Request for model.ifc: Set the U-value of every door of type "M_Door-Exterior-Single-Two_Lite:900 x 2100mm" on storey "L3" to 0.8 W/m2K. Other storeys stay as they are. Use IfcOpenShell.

First a look at what the model holds.

```python
import ifcopenshell
import ifcopenshell.util.element

model = ifcopenshell.open("model.ifc")
print(model.schema)
storey = next(s for s in model.by_type("IfcBuildingStorey") if s.Name == "L3")
doors = [e for e in ifcopenshell.util.element.get_decomposition(storey) if e.is_a("IfcDoor")]
seen = {}
for e in doors:
    element_type = ifcopenshell.util.element.get_type(e)
    key = (element_type.Name if element_type != e and element_type else None, ifcopenshell.util.element.get_pset(e, "Pset_DoorCommon", "ThermalTransmittance"))
    seen[key] = seen.get(key, 0) + 1
for (name, value), count in sorted(seen.items(), key=str):
    print(count, "x", name, "|", value)
```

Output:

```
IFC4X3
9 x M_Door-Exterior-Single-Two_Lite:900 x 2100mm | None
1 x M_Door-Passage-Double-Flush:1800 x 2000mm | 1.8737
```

```python
import ifcopenshell
import ifcopenshell.api.pset
import ifcopenshell.util.element

model = ifcopenshell.open("model.ifc")

storey = next(s for s in model.by_type("IfcBuildingStorey") if s.Name == "L3")
doors = [e for e in ifcopenshell.util.element.get_decomposition(storey) if e.is_a("IfcDoor")]

count = 0
for e in doors:
    element_type = ifcopenshell.util.element.get_type(e)
    if element_type in (None, e) or element_type.Name != "M_Door-Exterior-Single-Two_Lite:900 x 2100mm":
        continue
    # add_pset returns the element's existing set when there is one.
    pset = ifcopenshell.api.pset.add_pset(model, product=e, name="Pset_DoorCommon")
    ifcopenshell.api.pset.edit_pset(model, pset=pset, properties={"ThermalTransmittance": 0.8})
    count += 1

print(count, "doors updated")

model.write("model_rev.ifc")
```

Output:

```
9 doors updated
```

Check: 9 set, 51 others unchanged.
